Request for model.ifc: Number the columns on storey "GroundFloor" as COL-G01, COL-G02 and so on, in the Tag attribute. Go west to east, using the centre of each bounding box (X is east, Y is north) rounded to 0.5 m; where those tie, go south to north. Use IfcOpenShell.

First a look at what the model holds.

```python
import ifcopenshell
import ifcopenshell.util.element
import ifcopenshell.util.placement

model = ifcopenshell.open("model.ifc")
print(model.schema)
storey = next(s for s in model.by_type("IfcBuildingStorey") if s.Name == "GroundFloor")
columns = [e for e in ifcopenshell.util.element.get_decomposition(storey) if e.is_a("IfcColumn")]
for e in sorted(columns, key=lambda e: e.id()):
    origin = ifcopenshell.util.placement.get_local_placement(e.ObjectPlacement)[:3, 3]
    print(e.id(), e.Tag, e.Name, origin.round(2) + 0.0, sep=" | ")
```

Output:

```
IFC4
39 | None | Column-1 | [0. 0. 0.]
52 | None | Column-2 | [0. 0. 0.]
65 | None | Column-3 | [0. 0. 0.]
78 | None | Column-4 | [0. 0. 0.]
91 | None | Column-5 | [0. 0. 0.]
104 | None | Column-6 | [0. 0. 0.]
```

```python
import ifcopenshell
import ifcopenshell.geom
import ifcopenshell.util.element
import ifcopenshell.util.shape

model = ifcopenshell.open("model.ifc")
settings = ifcopenshell.geom.settings()
settings.set("use-world-coords", True)


def centre(element):
    shape = ifcopenshell.geom.create_shape(settings, element)
    return ifcopenshell.util.shape.get_bbox_centroid(shape.geometry)


storey = next(s for s in model.by_type("IfcBuildingStorey") if s.Name == "GroundFloor")
columns = [e for e in ifcopenshell.util.element.get_decomposition(storey) if e.is_a("IfcColumn")]

# Insertion points can sit at a corner or the storey origin, so sort by the geometry (in metres).
centres = {e: centre(e) for e in columns}
columns.sort(key=lambda e: (round(centres[e][0] / 0.5), centres[e][1]))

for i, e in enumerate(columns, start=1):
    number = f"COL-G{i:02d}"
    e.Tag = number
    print(e.id(), number)

model.write("model_v2.ifc")
```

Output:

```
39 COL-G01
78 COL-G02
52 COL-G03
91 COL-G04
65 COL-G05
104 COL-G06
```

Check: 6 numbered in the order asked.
